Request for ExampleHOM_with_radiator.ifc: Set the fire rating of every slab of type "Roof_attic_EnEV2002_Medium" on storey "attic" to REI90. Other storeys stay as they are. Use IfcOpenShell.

First a look at what the model holds.

```python
import ifcopenshell
import ifcopenshell.util.element

model = ifcopenshell.open("ExampleHOM_with_radiator.ifc")
print(model.schema)
storey = next(s for s in model.by_type("IfcBuildingStorey") if s.Name == "attic")
slabs = [e for e in ifcopenshell.util.element.get_decomposition(storey) if e.is_a("IfcSlab")]
seen = {}
for e in slabs:
    element_type = ifcopenshell.util.element.get_type(e)
    key = (element_type.Name if element_type != e and element_type else None, ifcopenshell.util.element.get_pset(e, "Pset_SlabCommon", "FireRating"))
    seen[key] = seen.get(key, 0) + 1
for (name, value), count in sorted(seen.items(), key=str):
    print(count, "x", name, "|", value)
```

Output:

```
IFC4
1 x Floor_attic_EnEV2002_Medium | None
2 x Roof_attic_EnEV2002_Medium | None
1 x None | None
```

```python
import ifcopenshell
import ifcopenshell.api.pset
import ifcopenshell.util.element

model = ifcopenshell.open("ExampleHOM_with_radiator.ifc")

storey = next(s for s in model.by_type("IfcBuildingStorey") if s.Name == "attic")
slabs = [e for e in ifcopenshell.util.element.get_decomposition(storey) if e.is_a("IfcSlab")]

count = 0
for e in slabs:
    element_type = ifcopenshell.util.element.get_type(e)
    if element_type in (None, e) or element_type.Name != "Roof_attic_EnEV2002_Medium":
        continue
    # add_pset returns the element's existing set when there is one.
    pset = ifcopenshell.api.pset.add_pset(model, product=e, name="Pset_SlabCommon")
    ifcopenshell.api.pset.edit_pset(model, pset=pset, properties={"FireRating": "REI90"})
    count += 1

print(count, "slabs updated")

model.write("ExampleHOM_with_radiator-out.ifc")
```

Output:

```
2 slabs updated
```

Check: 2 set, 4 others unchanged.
